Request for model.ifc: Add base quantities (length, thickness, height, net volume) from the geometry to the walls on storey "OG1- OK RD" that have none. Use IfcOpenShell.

First a look at what the model holds.

```python
import ifcopenshell
import ifcopenshell.util.element
import ifcopenshell.util.unit

model = ifcopenshell.open("model.ifc")
print(model.schema)
for unit_type in ("LENGTHUNIT", "AREAUNIT", "VOLUMEUNIT"):
    print(unit_type, ifcopenshell.util.unit.calculate_unit_scale(model, unit_type))
storey = next(s for s in model.by_type("IfcBuildingStorey") if s.Name == "OG1- OK RD")
walls = [e for e in ifcopenshell.util.element.get_decomposition(storey) if e.is_a("IfcWall")]
for e in sorted(walls, key=lambda e: e.id()):
    print(e.id(), e.is_a(), e.Name, list(ifcopenshell.util.element.get_psets(e, qtos_only=True)), sep=" | ")
```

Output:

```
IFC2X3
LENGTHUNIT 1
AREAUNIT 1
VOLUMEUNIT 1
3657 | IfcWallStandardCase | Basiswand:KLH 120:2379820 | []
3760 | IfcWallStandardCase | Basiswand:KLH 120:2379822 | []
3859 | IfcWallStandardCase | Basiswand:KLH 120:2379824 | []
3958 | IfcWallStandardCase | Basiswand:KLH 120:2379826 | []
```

```python
import ifcopenshell
import ifcopenshell.api.pset
import ifcopenshell.geom
import ifcopenshell.util.element
import ifcopenshell.util.shape
import ifcopenshell.util.unit

model = ifcopenshell.open("model.ifc")
unit_scale = ifcopenshell.util.unit.calculate_unit_scale(model)
volume_scale = ifcopenshell.util.unit.calculate_unit_scale(model, "VOLUMEUNIT")
settings = ifcopenshell.geom.settings()

storey = next(s for s in model.by_type("IfcBuildingStorey") if s.Name == "OG1- OK RD")
walls = [e for e in ifcopenshell.util.element.get_decomposition(storey) if e.is_a("IfcWall")]

for e in sorted(walls, key=lambda e: e.id()):
    if ifcopenshell.util.element.get_psets(e, qtos_only=True, should_inherit=False):
        continue
    # Geometry comes back in metres, in the element's own axes.
    shape = ifcopenshell.geom.create_shape(settings, e)
    values = {
        "Length": ifcopenshell.util.shape.get_x(shape.geometry) / unit_scale,
        "Width": ifcopenshell.util.shape.get_y(shape.geometry) / unit_scale,
        "Height": ifcopenshell.util.shape.get_z(shape.geometry) / unit_scale,
        "NetVolume": ifcopenshell.util.shape.get_volume(shape.geometry) / volume_scale,
    }
    qto = ifcopenshell.api.pset.add_qto(model, product=e, name="BaseQuantities")
    ifcopenshell.api.pset.edit_qto(model, qto=qto, properties=values)
    print(e.id(), {k: round(v, 3) for k, v in values.items()})

model.write("model_updated.ifc")
```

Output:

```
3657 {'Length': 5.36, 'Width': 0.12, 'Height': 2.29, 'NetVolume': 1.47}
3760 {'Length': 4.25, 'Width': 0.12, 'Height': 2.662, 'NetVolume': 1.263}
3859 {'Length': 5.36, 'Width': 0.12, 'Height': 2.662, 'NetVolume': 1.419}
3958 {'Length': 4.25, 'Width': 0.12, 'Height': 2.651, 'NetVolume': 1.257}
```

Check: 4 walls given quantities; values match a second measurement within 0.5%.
